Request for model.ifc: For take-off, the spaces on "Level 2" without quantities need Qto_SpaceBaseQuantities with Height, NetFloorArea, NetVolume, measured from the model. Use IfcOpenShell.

First a look at what the model holds.

```python
import ifcopenshell
import ifcopenshell.util.element
import ifcopenshell.util.unit

model = ifcopenshell.open("model.ifc")
print(model.schema)
for unit_type in ("LENGTHUNIT", "AREAUNIT", "VOLUMEUNIT"):
    print(unit_type, ifcopenshell.util.unit.calculate_unit_scale(model, unit_type))
storey = next(s for s in model.by_type("IfcBuildingStorey") if s.Name == "Level 2")
spaces = [e for e in ifcopenshell.util.element.get_decomposition(storey) if e.is_a("IfcSpace")]
for e in sorted(spaces, key=lambda e: e.id()):
    print(e.id(), e.is_a(), e.Name, list(ifcopenshell.util.element.get_psets(e, qtos_only=True)), sep=" | ")
```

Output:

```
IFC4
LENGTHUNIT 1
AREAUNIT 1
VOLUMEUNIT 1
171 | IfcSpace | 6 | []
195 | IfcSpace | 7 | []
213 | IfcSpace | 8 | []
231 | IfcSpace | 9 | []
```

```python
import ifcopenshell
import ifcopenshell.api.pset
import ifcopenshell.geom
import ifcopenshell.util.element
import ifcopenshell.util.shape
import ifcopenshell.util.unit

model = ifcopenshell.open("model.ifc")
unit_scale = ifcopenshell.util.unit.calculate_unit_scale(model)
area_scale = ifcopenshell.util.unit.calculate_unit_scale(model, "AREAUNIT")
volume_scale = ifcopenshell.util.unit.calculate_unit_scale(model, "VOLUMEUNIT")
settings = ifcopenshell.geom.settings()

storey = next(s for s in model.by_type("IfcBuildingStorey") if s.Name == "Level 2")
spaces = [e for e in ifcopenshell.util.element.get_decomposition(storey) if e.is_a("IfcSpace")]

for e in sorted(spaces, key=lambda e: e.id()):
    if ifcopenshell.util.element.get_psets(e, qtos_only=True, should_inherit=False):
        continue
    # Geometry comes back in metres, in the element's own axes.
    shape = ifcopenshell.geom.create_shape(settings, e)
    values = {
        "Height": ifcopenshell.util.shape.get_z(shape.geometry) / unit_scale,
        "NetFloorArea": ifcopenshell.util.shape.get_footprint_area(shape.geometry) / area_scale,
        "NetVolume": ifcopenshell.util.shape.get_volume(shape.geometry) / volume_scale,
    }
    qto = ifcopenshell.api.pset.add_qto(model, product=e, name="Qto_SpaceBaseQuantities")
    ifcopenshell.api.pset.edit_qto(model, qto=qto, properties=values)
    print(e.id(), {k: round(v, 3) for k, v in values.items()})

model.write("model_rev.ifc")
```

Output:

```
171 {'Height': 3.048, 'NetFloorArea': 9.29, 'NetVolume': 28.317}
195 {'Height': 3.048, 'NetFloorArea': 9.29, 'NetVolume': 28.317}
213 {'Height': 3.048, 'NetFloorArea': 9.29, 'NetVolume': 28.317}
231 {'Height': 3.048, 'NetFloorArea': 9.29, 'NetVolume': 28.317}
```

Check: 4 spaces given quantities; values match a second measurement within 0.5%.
